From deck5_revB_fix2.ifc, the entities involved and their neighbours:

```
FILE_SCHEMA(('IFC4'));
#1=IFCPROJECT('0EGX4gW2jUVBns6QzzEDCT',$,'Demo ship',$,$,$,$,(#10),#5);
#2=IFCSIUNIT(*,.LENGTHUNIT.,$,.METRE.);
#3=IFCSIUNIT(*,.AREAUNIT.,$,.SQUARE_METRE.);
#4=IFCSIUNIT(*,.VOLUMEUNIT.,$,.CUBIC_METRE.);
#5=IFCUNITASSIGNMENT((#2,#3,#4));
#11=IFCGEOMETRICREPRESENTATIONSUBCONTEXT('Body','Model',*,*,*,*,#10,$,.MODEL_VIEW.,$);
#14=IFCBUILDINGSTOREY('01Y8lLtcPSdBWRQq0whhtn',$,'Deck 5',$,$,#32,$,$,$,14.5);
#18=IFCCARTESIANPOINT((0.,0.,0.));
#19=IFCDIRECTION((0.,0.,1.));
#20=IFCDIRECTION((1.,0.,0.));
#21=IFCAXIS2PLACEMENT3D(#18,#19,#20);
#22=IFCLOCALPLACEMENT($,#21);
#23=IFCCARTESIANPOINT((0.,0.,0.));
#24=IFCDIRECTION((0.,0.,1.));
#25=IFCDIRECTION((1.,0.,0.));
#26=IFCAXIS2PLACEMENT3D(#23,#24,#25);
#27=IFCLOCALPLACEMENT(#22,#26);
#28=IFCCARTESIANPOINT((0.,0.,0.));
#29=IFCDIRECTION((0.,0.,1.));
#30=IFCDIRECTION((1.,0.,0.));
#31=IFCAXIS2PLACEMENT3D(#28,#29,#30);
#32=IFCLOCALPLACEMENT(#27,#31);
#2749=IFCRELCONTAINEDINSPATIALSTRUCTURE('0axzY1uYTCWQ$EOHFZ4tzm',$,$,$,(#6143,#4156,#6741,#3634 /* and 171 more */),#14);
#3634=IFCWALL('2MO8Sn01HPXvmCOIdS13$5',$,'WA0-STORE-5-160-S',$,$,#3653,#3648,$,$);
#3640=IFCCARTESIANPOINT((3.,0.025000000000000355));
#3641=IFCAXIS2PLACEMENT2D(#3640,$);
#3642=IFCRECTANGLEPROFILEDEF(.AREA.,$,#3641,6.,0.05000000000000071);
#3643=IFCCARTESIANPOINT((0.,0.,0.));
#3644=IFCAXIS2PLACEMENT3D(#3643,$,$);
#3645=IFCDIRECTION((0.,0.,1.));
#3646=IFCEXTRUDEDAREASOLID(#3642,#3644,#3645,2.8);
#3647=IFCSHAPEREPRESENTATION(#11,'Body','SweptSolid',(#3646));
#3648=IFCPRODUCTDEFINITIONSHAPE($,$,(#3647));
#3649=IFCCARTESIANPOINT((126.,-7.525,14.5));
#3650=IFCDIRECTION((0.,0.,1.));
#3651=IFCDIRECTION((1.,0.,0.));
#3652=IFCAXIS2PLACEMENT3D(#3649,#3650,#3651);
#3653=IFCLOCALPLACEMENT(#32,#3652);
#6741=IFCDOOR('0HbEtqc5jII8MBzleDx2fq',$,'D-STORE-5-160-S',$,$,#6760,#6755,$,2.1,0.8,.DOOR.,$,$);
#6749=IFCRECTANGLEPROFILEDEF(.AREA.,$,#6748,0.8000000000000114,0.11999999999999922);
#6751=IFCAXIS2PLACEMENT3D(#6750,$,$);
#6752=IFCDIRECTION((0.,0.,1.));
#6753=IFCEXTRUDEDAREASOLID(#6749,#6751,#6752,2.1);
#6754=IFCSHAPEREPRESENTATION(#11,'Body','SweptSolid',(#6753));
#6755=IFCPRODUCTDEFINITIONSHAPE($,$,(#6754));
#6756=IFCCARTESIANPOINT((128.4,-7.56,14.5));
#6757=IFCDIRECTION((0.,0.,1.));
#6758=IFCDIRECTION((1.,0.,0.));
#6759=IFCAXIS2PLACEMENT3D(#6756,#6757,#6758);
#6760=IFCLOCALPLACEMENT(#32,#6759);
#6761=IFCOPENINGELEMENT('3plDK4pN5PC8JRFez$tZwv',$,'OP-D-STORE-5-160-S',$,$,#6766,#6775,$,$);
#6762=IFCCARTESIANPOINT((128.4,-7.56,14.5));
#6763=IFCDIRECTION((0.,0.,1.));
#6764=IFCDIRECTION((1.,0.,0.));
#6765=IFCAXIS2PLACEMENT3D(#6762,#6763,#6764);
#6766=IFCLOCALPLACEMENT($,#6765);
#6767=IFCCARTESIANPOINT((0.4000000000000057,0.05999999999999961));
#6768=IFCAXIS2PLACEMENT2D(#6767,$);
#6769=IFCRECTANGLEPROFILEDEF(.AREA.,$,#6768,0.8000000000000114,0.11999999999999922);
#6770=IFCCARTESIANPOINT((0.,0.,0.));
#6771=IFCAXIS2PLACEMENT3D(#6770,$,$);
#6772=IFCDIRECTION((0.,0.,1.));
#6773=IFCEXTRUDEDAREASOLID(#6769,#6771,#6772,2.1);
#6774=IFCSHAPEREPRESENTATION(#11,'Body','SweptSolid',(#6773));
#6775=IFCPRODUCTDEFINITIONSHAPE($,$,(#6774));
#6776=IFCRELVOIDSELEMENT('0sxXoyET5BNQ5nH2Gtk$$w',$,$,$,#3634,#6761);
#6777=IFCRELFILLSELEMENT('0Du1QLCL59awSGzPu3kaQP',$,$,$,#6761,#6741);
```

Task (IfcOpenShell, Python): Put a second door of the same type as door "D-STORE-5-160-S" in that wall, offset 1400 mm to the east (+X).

```python
import ifcopenshell
import ifcopenshell.api.feature
import ifcopenshell.api.geometry
import ifcopenshell.api.root
import ifcopenshell.geom
import ifcopenshell.util.element
import ifcopenshell.util.placement
import ifcopenshell.util.shape
import ifcopenshell.util.unit

model = ifcopenshell.open("deck5_revB_fix2.ifc")
unit_scale = ifcopenshell.util.unit.calculate_unit_scale(model)
settings = ifcopenshell.geom.settings()


def volume(element):
    """Net volume in cubic metres, openings subtracted."""
    shape = ifcopenshell.geom.create_shape(settings, element)
    return ifcopenshell.util.shape.get_volume(shape.geometry)


door = model.by_id(6741)
opening = door.FillsVoids[0].RelatingOpeningElement
wall = opening.VoidsElements[0].RelatingBuildingElement
before = volume(wall)
shift = ifcopenshell.util.placement.get_local_placement(wall.ObjectPlacement)[:3, 0] * 1.4 / unit_scale

# copy_class copies the void relationship, type, container and properties, but no geometry.
new_opening = ifcopenshell.api.root.copy_class(model, product=opening)
new_opening.Representation = ifcopenshell.util.element.copy_deep(
    model, opening.Representation, exclude=["IfcGeometricRepresentationContext", "IfcRepresentationMap"]
)
new_door = ifcopenshell.api.root.copy_class(model, product=door)
new_door.Representation = ifcopenshell.util.element.copy_deep(
    model, door.Representation, exclude=["IfcGeometricRepresentationContext", "IfcRepresentationMap"]
)
ifcopenshell.api.feature.add_filling(model, opening=new_opening, element=new_door)

for old, new in ((opening, new_opening), (door, new_door)):
    matrix = ifcopenshell.util.placement.get_local_placement(old.ObjectPlacement)
    matrix[:3, 3] += shift
    ifcopenshell.api.geometry.edit_object_placement(model, product=new, matrix=matrix, is_si=False)

after = volume(wall)

print(f"wall volume {before:.3f} -> {after:.3f} m3")

model.write("deck5_revB_fix2_v2.ifc")
```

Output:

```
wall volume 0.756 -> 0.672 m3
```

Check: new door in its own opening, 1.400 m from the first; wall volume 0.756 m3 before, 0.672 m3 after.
